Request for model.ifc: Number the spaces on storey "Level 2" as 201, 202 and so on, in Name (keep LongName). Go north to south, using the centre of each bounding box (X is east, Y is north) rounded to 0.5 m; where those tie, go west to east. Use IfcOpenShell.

First a look at what the model holds.

```python
import ifcopenshell
import ifcopenshell.util.element
import ifcopenshell.util.placement

model = ifcopenshell.open("model.ifc")
print(model.schema)
storey = next(s for s in model.by_type("IfcBuildingStorey") if s.Name == "Level 2")
spaces = [e for e in ifcopenshell.util.element.get_decomposition(storey) if e.is_a("IfcSpace")]
for e in sorted(spaces, key=lambda e: e.id()):
    origin = ifcopenshell.util.placement.get_local_placement(e.ObjectPlacement)[:3, 3]
    print(e.id(), e.Name, e.LongName, origin.round(2) + 0.0, sep=" | ")
```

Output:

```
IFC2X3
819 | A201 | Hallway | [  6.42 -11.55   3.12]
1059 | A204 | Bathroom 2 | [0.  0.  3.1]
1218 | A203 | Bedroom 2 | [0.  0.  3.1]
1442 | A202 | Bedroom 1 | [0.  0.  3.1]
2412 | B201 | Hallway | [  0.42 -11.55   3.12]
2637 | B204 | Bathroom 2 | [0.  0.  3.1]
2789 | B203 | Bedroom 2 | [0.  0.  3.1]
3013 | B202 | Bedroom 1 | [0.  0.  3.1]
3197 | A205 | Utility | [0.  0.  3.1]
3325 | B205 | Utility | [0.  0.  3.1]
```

```python
import ifcopenshell
import ifcopenshell.geom
import ifcopenshell.util.element
import ifcopenshell.util.shape

model = ifcopenshell.open("model.ifc")
settings = ifcopenshell.geom.settings()
settings.set("use-world-coords", True)


def centre(element):
    shape = ifcopenshell.geom.create_shape(settings, element)
    return ifcopenshell.util.shape.get_bbox_centroid(shape.geometry)


storey = next(s for s in model.by_type("IfcBuildingStorey") if s.Name == "Level 2")
spaces = [e for e in ifcopenshell.util.element.get_decomposition(storey) if e.is_a("IfcSpace")]

# Insertion points can sit at a corner or the storey origin, so sort by the geometry (in metres).
centres = {e: centre(e) for e in spaces}
spaces.sort(key=lambda e: (-round(centres[e][1] / 0.5), centres[e][0]))

for i, e in enumerate(spaces, start=1):
    number = f"2{i:02d}"
    e.Name = number
    print(e.id(), number)

model.write("model_v2.ifc")
```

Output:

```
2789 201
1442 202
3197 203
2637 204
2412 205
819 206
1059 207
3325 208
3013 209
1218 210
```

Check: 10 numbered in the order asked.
